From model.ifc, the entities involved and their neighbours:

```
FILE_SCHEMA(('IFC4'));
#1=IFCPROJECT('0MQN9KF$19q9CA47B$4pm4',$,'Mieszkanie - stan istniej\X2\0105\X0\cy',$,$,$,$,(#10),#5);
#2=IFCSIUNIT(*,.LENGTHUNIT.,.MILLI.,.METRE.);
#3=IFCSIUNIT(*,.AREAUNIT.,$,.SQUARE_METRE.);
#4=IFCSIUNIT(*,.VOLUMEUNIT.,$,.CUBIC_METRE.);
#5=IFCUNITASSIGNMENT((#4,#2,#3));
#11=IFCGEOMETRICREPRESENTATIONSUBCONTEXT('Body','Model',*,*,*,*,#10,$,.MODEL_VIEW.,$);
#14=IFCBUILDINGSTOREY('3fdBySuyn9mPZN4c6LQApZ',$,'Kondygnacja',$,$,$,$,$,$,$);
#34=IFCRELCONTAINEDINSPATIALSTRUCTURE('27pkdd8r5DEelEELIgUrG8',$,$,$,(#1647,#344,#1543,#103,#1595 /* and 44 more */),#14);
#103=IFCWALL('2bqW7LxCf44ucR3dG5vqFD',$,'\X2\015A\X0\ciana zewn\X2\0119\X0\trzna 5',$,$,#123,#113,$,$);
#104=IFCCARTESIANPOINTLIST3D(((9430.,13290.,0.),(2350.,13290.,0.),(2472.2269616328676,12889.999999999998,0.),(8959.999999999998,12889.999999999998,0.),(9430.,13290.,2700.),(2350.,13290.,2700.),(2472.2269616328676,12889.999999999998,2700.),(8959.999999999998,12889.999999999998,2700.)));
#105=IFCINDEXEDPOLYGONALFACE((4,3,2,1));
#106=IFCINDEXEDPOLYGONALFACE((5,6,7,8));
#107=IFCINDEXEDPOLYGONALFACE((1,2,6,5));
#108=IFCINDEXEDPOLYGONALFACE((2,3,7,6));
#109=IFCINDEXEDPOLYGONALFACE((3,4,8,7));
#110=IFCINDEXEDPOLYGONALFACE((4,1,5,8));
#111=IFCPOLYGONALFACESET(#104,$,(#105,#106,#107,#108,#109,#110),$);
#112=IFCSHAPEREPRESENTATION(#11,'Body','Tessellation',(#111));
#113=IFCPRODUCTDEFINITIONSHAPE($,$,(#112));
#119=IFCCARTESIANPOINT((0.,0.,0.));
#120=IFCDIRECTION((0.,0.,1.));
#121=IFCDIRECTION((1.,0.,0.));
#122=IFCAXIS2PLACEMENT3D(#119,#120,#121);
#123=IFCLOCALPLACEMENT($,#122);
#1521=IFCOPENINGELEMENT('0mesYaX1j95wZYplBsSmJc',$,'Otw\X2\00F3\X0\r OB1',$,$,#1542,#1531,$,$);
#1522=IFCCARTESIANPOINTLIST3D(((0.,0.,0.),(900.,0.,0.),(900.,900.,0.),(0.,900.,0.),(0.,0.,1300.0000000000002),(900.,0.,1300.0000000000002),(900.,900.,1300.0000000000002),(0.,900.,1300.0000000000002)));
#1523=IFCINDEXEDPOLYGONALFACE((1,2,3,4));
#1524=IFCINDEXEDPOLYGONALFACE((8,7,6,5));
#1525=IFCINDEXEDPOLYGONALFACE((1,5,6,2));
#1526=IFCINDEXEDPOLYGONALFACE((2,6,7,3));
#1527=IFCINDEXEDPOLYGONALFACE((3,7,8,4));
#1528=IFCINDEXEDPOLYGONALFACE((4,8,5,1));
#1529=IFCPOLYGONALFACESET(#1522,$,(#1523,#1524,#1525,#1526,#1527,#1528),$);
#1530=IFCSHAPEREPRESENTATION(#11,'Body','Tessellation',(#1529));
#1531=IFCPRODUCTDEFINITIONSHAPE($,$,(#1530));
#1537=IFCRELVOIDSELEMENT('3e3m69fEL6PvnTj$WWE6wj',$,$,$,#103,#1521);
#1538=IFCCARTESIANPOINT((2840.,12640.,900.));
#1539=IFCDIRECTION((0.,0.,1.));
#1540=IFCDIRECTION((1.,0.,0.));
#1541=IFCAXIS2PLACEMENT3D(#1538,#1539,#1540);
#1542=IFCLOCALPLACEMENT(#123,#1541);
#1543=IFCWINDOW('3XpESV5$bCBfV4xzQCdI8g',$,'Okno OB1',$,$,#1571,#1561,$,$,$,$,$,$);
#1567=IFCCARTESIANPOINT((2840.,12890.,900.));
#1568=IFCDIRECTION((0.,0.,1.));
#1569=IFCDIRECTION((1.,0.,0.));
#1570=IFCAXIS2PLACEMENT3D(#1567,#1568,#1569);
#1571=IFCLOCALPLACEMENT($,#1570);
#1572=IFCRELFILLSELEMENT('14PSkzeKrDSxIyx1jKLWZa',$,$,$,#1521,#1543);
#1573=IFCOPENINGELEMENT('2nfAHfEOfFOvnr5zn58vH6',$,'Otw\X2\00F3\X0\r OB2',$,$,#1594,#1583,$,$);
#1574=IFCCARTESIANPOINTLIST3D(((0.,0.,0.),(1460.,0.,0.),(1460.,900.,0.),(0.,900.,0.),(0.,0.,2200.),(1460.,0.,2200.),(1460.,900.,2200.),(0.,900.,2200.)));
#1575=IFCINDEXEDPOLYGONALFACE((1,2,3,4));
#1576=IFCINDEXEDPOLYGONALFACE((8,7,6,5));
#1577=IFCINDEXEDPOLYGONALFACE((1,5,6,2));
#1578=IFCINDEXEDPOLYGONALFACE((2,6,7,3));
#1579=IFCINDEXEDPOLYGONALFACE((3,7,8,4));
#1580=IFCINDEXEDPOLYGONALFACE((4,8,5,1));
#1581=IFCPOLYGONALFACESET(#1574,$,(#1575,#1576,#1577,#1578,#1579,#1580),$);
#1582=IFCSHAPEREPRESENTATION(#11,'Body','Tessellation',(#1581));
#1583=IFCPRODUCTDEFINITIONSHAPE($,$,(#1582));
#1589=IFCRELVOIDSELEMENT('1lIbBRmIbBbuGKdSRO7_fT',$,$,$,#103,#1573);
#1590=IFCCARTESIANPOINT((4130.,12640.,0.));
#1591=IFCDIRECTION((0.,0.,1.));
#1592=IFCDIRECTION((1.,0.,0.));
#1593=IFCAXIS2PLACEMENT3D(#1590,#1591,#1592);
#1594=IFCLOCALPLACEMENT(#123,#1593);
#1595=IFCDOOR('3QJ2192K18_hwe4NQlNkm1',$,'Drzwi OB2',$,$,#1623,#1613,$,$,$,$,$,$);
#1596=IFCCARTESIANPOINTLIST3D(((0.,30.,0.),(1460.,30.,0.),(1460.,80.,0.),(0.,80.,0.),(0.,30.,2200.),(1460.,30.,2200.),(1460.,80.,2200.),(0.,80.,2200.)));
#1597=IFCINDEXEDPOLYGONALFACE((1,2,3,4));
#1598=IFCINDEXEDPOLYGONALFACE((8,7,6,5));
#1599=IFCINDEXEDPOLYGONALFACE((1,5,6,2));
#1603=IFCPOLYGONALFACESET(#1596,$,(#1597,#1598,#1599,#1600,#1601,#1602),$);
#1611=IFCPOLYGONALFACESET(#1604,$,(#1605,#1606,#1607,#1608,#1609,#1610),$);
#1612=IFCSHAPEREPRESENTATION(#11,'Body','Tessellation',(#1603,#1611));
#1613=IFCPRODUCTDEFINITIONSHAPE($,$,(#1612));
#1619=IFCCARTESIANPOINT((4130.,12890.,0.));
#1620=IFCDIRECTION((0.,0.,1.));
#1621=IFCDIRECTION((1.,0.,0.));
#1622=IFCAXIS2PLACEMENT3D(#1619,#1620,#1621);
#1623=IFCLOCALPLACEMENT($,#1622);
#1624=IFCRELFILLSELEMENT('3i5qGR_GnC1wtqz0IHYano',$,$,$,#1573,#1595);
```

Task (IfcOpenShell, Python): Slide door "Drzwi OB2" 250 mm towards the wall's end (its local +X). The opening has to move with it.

```python
import ifcopenshell
import ifcopenshell.api.geometry
import ifcopenshell.util.placement

model = ifcopenshell.open("model.ifc")

door = model.by_id(1595)
opening = door.FillsVoids[0].RelatingOpeningElement
wall = opening.VoidsElements[0].RelatingBuildingElement

wall_matrix = ifcopenshell.util.placement.get_local_placement(wall.ObjectPlacement)
shift = wall_matrix[:3, 0] * 250.0
before = ifcopenshell.util.placement.get_local_placement(door.ObjectPlacement)[:3, 3].copy()

# The door is not placed relative to its opening, so move both.
for product in (opening, door):
    matrix = ifcopenshell.util.placement.get_local_placement(product.ObjectPlacement)
    matrix[:3, 3] += shift
    ifcopenshell.api.geometry.edit_object_placement(model, product=product, matrix=matrix, is_si=False)

after = ifcopenshell.util.placement.get_local_placement(door.ObjectPlacement)[:3, 3]
print("door moved by", (after - before).round(3) + 0.0)

model.write("model-out.ifc")
```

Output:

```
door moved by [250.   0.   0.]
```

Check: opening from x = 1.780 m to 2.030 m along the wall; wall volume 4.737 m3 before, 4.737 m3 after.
